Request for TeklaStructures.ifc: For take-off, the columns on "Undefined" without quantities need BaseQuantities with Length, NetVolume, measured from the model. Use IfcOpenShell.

First a look at what the model holds.

```python
import ifcopenshell
import ifcopenshell.util.element
import ifcopenshell.util.unit

model = ifcopenshell.open("TeklaStructures.ifc")
print(model.schema)
for unit_type in ("LENGTHUNIT", "AREAUNIT", "VOLUMEUNIT"):
    print(unit_type, ifcopenshell.util.unit.calculate_unit_scale(model, unit_type))
storey = next(s for s in model.by_type("IfcBuildingStorey") if s.Name == "Undefined")
columns = [e for e in ifcopenshell.util.element.get_decomposition(storey) if e.is_a("IfcColumn")]
for e in sorted(columns, key=lambda e: e.id()):
    print(e.id(), e.is_a(), e.Name, list(ifcopenshell.util.element.get_psets(e, qtos_only=True)), sep=" | ")
```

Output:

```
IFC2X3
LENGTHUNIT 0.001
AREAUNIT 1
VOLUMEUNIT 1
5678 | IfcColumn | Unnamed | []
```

```python
import ifcopenshell
import ifcopenshell.api.pset
import ifcopenshell.geom
import ifcopenshell.util.element
import ifcopenshell.util.shape
import ifcopenshell.util.unit

model = ifcopenshell.open("TeklaStructures.ifc")
unit_scale = ifcopenshell.util.unit.calculate_unit_scale(model)
volume_scale = ifcopenshell.util.unit.calculate_unit_scale(model, "VOLUMEUNIT")
settings = ifcopenshell.geom.settings()

storey = next(s for s in model.by_type("IfcBuildingStorey") if s.Name == "Undefined")
columns = [e for e in ifcopenshell.util.element.get_decomposition(storey) if e.is_a("IfcColumn")]

for e in sorted(columns, key=lambda e: e.id()):
    if ifcopenshell.util.element.get_psets(e, qtos_only=True, should_inherit=False):
        continue
    # Geometry comes back in metres, in the element's own axes.
    shape = ifcopenshell.geom.create_shape(settings, e)
    values = {
        "Length": ifcopenshell.util.shape.get_z(shape.geometry) / unit_scale,
        "NetVolume": ifcopenshell.util.shape.get_volume(shape.geometry) / volume_scale,
    }
    qto = ifcopenshell.api.pset.add_qto(model, product=e, name="BaseQuantities")
    ifcopenshell.api.pset.edit_qto(model, qto=qto, properties=values)
    print(e.id(), {k: round(v, 3) for k, v in values.items()})

model.write("TeklaStructures_v2.ifc")
```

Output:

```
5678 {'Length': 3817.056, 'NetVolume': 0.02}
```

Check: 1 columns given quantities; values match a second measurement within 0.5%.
